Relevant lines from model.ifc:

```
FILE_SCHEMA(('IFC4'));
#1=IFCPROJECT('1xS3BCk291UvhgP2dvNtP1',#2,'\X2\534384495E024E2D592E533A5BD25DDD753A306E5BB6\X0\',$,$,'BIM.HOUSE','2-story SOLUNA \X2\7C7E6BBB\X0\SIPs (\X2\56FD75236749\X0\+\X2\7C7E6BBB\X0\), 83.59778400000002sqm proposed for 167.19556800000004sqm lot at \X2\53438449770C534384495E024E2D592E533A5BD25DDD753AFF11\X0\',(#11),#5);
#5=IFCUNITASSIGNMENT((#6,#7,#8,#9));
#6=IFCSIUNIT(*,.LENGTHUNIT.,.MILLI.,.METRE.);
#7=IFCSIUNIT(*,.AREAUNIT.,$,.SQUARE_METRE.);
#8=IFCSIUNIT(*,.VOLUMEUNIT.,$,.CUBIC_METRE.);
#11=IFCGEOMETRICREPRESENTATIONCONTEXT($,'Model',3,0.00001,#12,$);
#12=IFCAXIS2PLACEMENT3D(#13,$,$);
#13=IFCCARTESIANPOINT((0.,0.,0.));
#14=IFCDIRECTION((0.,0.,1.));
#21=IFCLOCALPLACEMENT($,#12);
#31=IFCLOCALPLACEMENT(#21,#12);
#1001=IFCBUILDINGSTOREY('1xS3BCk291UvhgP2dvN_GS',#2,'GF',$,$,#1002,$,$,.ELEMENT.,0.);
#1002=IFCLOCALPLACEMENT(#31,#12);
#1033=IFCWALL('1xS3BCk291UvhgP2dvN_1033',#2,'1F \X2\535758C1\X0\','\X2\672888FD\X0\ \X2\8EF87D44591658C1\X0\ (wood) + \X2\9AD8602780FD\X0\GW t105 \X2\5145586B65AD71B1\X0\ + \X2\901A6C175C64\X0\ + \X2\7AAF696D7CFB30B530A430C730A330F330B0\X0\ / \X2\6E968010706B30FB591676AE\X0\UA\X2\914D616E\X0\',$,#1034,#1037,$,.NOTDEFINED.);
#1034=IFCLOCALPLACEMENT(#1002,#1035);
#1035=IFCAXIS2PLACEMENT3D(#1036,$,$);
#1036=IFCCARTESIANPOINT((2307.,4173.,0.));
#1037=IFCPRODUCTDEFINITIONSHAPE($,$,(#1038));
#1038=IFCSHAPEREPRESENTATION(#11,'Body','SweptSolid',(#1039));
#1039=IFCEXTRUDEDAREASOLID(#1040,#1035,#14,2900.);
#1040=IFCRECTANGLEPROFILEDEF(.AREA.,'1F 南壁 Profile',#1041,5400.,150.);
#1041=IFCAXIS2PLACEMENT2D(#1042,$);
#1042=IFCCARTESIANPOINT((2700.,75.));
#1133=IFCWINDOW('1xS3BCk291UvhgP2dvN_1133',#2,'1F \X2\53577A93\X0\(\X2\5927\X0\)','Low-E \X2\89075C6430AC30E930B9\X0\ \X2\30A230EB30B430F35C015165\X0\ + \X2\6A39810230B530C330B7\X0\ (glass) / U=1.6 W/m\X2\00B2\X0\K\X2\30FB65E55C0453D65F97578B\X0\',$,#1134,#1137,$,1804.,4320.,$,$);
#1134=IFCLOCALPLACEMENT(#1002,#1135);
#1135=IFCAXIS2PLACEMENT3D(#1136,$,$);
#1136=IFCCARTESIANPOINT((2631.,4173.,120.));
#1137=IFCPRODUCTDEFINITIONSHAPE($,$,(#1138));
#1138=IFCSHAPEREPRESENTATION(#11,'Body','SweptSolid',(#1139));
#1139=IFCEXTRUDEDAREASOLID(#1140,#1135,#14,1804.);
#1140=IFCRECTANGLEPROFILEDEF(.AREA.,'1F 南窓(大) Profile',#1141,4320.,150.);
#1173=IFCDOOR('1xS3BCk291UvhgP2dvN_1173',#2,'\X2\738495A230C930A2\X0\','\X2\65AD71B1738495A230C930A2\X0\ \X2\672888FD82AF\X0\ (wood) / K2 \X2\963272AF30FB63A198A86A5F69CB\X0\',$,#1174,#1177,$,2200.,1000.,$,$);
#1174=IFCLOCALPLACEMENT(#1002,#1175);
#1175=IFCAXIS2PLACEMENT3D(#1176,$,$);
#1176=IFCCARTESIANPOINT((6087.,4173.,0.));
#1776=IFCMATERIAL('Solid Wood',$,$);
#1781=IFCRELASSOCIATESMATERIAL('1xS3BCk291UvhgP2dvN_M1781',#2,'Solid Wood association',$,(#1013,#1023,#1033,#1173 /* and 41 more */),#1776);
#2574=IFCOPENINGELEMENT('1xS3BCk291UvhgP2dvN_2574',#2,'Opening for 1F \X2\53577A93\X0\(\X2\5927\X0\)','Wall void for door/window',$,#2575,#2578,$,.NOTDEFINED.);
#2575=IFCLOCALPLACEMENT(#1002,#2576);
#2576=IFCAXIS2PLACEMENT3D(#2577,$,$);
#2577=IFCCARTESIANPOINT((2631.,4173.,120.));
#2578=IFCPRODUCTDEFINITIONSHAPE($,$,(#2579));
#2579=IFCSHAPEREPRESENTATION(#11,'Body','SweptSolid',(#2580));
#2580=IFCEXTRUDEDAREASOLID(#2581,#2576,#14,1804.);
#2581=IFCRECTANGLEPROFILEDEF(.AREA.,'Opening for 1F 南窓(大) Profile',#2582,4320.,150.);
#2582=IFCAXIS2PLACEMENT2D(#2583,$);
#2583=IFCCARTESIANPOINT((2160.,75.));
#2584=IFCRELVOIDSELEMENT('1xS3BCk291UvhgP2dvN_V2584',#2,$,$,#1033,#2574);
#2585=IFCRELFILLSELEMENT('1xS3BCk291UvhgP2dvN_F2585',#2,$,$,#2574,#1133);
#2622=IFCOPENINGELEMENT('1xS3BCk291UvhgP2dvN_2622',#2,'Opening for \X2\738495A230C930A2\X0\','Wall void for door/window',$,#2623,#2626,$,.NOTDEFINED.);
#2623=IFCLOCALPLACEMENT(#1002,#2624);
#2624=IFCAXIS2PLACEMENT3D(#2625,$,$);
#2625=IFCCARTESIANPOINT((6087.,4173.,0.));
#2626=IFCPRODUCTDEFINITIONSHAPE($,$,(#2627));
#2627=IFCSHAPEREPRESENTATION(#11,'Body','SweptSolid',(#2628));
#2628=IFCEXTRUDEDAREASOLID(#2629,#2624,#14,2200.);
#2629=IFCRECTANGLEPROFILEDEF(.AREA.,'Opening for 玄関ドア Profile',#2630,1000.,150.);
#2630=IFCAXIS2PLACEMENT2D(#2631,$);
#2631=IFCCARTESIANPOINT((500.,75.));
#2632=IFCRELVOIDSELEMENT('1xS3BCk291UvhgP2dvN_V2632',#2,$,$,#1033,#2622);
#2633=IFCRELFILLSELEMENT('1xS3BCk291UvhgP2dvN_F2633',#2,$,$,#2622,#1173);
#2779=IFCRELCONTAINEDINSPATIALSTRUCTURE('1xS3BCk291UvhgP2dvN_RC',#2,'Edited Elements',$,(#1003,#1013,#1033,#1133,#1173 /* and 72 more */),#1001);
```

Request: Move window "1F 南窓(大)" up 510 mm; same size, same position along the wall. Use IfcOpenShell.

```python
import numpy as np
import ifcopenshell
import ifcopenshell.api.geometry
import ifcopenshell.util.placement
import ifcopenshell.util.unit

model = ifcopenshell.open("model.ifc")
unit_scale = ifcopenshell.util.unit.calculate_unit_scale(model)

window = model.by_guid("1xS3BCk291UvhgP2dvN_1133")
opening = window.FillsVoids[0].RelatingOpeningElement
dz = 510.0

shift = np.array([0.0, 0.0, dz])
# The window is not placed relative to its opening, so move both.
for product in (opening, window):
    matrix = ifcopenshell.util.placement.get_local_placement(product.ObjectPlacement)
    matrix[:3, 3] += shift
    ifcopenshell.api.geometry.edit_object_placement(model, product=product, matrix=matrix, is_si=False)

print(f"moved by {dz * unit_scale:+.3f} m")

model.write("model-out.ifc")
```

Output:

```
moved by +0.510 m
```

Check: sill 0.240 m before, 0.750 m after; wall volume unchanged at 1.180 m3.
